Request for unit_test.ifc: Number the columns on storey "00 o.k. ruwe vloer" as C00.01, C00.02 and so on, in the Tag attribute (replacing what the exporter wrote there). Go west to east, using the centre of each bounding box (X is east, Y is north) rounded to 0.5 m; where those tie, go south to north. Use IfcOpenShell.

First a look at what the model holds.

```python
import ifcopenshell
import ifcopenshell.util.element
import ifcopenshell.util.placement

model = ifcopenshell.open("unit_test.ifc")
print(model.schema)
storey = next(s for s in model.by_type("IfcBuildingStorey") if s.Name == "00 o.k. ruwe vloer")
columns = [e for e in ifcopenshell.util.element.get_decomposition(storey) if e.is_a("IfcColumn")]
for e in sorted(columns, key=lambda e: e.id()):
    origin = ifcopenshell.util.placement.get_local_placement(e.ObjectPlacement)[:3, 3]
    print(e.id(), e.Tag, e.Name, origin.round(2) + 0.0, sep=" | ")
```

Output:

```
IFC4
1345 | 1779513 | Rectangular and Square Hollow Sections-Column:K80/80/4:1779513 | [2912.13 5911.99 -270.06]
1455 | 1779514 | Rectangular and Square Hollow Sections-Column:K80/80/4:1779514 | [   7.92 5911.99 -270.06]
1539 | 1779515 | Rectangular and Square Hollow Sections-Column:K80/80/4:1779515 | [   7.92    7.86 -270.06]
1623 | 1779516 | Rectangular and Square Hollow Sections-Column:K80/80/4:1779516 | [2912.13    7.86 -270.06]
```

```python
import ifcopenshell
import ifcopenshell.geom
import ifcopenshell.util.element
import ifcopenshell.util.shape

model = ifcopenshell.open("unit_test.ifc")
settings = ifcopenshell.geom.settings()
settings.set("use-world-coords", True)


def centre(element):
    shape = ifcopenshell.geom.create_shape(settings, element)
    return ifcopenshell.util.shape.get_bbox_centroid(shape.geometry)


storey = next(s for s in model.by_type("IfcBuildingStorey") if s.Name == "00 o.k. ruwe vloer")
columns = [e for e in ifcopenshell.util.element.get_decomposition(storey) if e.is_a("IfcColumn")]

# Insertion points can sit at a corner or the storey origin, so sort by the geometry (in metres).
centres = {e: centre(e) for e in columns}
columns.sort(key=lambda e: (round(centres[e][0] / 0.5), centres[e][1]))

for i, e in enumerate(columns, start=1):
    number = f"C00.{i:02d}"
    e.Tag = number
    print(e.id(), number)

model.write("unit_test-out.ifc")
```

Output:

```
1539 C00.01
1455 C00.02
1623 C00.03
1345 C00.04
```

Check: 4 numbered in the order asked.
